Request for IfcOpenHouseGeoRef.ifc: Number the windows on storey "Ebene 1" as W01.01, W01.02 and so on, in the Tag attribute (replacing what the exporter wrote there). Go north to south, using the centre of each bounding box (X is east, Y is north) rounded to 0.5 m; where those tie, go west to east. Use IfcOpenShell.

First a look at what the model holds.

```python
import ifcopenshell
import ifcopenshell.util.element
import ifcopenshell.util.placement

model = ifcopenshell.open("IfcOpenHouseGeoRef.ifc")
print(model.schema)
storey = next(s for s in model.by_type("IfcBuildingStorey") if s.Name == "Ebene 1")
windows = [e for e in ifcopenshell.util.element.get_decomposition(storey) if e.is_a("IfcWindow")]
for e in sorted(windows, key=lambda e: e.id()):
    origin = ifcopenshell.util.placement.get_local_placement(e.ObjectPlacement)[:3, 3]
    print(e.id(), e.Tag, e.Name, origin.round(2) + 0.0, sep=" | ")
```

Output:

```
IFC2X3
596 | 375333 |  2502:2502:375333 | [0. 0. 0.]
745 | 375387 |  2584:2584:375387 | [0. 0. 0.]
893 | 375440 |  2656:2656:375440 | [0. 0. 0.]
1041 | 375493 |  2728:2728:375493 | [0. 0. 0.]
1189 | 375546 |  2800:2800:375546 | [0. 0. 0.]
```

```python
import ifcopenshell
import ifcopenshell.geom
import ifcopenshell.util.element
import ifcopenshell.util.shape

model = ifcopenshell.open("IfcOpenHouseGeoRef.ifc")
settings = ifcopenshell.geom.settings()
settings.set("use-world-coords", True)


def centre(element):
    shape = ifcopenshell.geom.create_shape(settings, element)
    return ifcopenshell.util.shape.get_bbox_centroid(shape.geometry)


storey = next(s for s in model.by_type("IfcBuildingStorey") if s.Name == "Ebene 1")
windows = [e for e in ifcopenshell.util.element.get_decomposition(storey) if e.is_a("IfcWindow")]

# Insertion points can sit at a corner or the storey origin, so sort by the geometry (in metres).
centres = {e: centre(e) for e in windows}
windows.sort(key=lambda e: (-round(centres[e][1] / 0.5), centres[e][0]))

for i, e in enumerate(windows, start=1):
    number = f"W01.{i:02d}"
    e.Tag = number
    print(e.id(), number)

model.write("IfcOpenHouseGeoRef_rev.ifc")
```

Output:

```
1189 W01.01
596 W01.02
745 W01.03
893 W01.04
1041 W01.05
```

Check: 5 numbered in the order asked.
